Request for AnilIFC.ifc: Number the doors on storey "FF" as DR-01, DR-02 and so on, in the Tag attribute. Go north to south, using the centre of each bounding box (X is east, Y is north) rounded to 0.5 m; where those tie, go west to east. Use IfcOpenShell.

First a look at what the model holds.

```python
import ifcopenshell
import ifcopenshell.util.element
import ifcopenshell.util.placement

model = ifcopenshell.open("AnilIFC.ifc")
print(model.schema)
storey = next(s for s in model.by_type("IfcBuildingStorey") if s.Name == "FF")
doors = [e for e in ifcopenshell.util.element.get_decomposition(storey) if e.is_a("IfcDoor")]
for e in sorted(doors, key=lambda e: e.id()):
    origin = ifcopenshell.util.placement.get_local_placement(e.ObjectPlacement)[:3, 3]
    print(e.id(), e.Tag, e.Name, origin.round(2) + 0.0, sep=" | ")
```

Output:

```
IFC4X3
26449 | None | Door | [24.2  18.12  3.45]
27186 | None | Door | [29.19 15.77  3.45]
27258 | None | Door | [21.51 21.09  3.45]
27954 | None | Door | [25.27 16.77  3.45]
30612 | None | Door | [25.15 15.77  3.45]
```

```python
import ifcopenshell
import ifcopenshell.geom
import ifcopenshell.util.element
import ifcopenshell.util.shape

model = ifcopenshell.open("AnilIFC.ifc")
settings = ifcopenshell.geom.settings()
settings.set("use-world-coords", True)


def centre(element):
    shape = ifcopenshell.geom.create_shape(settings, element)
    return ifcopenshell.util.shape.get_bbox_centroid(shape.geometry)


storey = next(s for s in model.by_type("IfcBuildingStorey") if s.Name == "FF")
doors = [e for e in ifcopenshell.util.element.get_decomposition(storey) if e.is_a("IfcDoor")]

# Insertion points can sit at a corner or the storey origin, so sort by the geometry (in metres).
centres = {e: centre(e) for e in doors}
doors.sort(key=lambda e: (-round(centres[e][1] / 0.5), centres[e][0]))

for i, e in enumerate(doors, start=1):
    number = f"DR-{i:02d}"
    e.Tag = number
    print(e.id(), number)

model.write("AnilIFC_v2.ifc")
```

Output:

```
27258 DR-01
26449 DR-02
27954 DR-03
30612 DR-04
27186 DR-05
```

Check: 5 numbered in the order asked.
